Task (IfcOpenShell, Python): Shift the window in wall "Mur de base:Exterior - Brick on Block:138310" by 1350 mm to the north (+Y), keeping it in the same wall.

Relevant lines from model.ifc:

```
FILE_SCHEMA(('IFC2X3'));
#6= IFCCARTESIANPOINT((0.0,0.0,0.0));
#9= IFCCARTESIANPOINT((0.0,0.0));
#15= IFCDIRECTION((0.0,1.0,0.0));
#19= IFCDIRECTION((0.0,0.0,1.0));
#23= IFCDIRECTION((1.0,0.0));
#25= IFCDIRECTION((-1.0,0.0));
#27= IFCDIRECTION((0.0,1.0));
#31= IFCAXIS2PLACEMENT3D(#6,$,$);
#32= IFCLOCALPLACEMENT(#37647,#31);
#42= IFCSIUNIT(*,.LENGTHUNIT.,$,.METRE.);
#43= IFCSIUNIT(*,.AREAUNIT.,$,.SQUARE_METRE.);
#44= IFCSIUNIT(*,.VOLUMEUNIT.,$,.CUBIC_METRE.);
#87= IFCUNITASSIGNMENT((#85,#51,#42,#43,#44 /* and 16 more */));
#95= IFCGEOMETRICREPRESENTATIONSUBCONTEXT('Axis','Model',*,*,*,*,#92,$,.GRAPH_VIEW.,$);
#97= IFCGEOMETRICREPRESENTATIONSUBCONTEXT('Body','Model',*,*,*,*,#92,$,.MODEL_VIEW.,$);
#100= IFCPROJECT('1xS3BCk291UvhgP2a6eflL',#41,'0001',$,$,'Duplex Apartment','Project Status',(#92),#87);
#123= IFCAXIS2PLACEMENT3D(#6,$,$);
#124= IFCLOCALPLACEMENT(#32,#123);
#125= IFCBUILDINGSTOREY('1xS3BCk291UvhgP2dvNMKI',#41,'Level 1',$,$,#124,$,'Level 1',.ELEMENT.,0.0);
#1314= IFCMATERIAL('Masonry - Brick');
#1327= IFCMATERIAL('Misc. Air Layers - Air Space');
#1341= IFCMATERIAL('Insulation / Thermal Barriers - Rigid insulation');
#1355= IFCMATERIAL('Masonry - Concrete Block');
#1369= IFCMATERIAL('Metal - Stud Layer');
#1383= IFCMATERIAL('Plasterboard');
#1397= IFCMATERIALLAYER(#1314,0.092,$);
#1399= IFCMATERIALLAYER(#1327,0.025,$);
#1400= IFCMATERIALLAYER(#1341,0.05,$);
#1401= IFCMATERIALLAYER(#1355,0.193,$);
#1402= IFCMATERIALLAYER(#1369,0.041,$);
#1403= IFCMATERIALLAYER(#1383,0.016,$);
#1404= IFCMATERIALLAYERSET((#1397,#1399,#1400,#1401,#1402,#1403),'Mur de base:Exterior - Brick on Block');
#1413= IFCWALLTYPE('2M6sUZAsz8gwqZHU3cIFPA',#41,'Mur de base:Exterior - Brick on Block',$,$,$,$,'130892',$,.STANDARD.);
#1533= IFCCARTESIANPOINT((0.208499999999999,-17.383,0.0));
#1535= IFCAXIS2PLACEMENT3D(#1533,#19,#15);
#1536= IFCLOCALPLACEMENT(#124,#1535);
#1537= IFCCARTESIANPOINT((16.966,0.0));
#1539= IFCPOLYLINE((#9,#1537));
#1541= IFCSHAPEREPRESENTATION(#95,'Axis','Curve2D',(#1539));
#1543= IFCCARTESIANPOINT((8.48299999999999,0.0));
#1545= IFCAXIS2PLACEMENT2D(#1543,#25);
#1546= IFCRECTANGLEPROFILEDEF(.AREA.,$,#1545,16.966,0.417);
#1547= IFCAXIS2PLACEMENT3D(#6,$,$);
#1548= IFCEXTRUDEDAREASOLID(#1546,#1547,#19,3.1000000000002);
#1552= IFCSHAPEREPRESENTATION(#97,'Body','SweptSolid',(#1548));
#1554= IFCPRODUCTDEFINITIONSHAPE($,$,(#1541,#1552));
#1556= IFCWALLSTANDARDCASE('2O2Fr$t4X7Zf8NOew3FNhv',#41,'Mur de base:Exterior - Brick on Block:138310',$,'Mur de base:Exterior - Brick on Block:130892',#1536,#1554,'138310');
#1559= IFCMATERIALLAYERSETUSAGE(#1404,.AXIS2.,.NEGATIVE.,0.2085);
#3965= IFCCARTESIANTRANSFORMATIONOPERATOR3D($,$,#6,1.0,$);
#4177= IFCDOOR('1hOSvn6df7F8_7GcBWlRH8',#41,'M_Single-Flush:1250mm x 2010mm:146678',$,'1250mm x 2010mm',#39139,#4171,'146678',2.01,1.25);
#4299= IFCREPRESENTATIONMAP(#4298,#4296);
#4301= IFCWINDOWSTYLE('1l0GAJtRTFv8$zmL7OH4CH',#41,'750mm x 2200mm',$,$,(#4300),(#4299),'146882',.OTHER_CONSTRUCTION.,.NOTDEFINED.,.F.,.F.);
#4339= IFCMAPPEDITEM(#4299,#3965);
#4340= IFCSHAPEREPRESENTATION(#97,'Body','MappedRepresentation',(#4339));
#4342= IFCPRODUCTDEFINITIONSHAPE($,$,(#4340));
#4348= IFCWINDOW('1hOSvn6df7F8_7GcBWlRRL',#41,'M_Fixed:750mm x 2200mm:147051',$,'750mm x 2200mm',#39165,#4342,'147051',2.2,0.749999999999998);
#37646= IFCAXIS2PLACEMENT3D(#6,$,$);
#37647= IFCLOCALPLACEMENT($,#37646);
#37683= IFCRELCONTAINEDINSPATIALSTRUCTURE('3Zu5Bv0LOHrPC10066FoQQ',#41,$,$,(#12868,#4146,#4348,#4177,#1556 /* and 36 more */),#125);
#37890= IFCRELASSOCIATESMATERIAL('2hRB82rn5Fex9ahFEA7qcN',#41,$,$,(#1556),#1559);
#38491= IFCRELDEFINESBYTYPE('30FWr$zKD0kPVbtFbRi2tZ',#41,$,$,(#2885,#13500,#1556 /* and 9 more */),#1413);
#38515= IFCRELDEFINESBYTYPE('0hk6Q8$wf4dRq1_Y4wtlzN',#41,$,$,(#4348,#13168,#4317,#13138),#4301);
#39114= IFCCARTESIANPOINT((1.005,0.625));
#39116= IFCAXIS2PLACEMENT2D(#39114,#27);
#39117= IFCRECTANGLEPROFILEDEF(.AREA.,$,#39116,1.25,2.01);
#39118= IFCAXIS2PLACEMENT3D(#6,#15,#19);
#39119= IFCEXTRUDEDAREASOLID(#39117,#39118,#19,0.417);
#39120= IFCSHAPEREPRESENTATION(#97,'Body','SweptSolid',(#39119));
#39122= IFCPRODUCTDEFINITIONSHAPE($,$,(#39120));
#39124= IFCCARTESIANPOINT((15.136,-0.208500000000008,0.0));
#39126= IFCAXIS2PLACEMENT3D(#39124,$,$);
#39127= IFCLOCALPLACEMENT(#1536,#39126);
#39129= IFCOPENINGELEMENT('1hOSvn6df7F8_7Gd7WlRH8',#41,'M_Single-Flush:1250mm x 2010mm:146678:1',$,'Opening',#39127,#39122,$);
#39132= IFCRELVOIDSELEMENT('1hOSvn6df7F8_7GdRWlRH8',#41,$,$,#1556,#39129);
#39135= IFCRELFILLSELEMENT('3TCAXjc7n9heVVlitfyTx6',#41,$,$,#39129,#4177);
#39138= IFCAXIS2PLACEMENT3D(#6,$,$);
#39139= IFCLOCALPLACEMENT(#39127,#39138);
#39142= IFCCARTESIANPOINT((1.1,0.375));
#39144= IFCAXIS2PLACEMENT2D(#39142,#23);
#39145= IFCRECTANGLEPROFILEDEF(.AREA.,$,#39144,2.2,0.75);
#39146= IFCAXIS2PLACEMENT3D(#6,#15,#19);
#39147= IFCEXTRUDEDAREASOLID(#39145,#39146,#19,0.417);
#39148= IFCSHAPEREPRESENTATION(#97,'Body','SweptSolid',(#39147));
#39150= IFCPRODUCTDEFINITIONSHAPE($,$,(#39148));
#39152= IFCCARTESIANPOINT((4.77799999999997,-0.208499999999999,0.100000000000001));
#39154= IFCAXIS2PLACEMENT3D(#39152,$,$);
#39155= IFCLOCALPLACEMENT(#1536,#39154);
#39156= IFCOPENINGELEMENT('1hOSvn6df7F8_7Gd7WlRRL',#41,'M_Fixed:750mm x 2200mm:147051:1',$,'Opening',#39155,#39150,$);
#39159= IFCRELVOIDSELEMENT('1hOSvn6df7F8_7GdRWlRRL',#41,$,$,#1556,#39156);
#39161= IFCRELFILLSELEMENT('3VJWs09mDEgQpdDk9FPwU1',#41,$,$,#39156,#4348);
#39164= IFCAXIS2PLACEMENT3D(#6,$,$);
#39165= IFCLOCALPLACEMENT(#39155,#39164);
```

```python
import ifcopenshell
import ifcopenshell.api.geometry
import ifcopenshell.util.placement

model = ifcopenshell.open("model.ifc")

window = model.by_guid("1hOSvn6df7F8_7GcBWlRRL")
opening = window.FillsVoids[0].RelatingOpeningElement
wall = opening.VoidsElements[0].RelatingBuildingElement

wall_matrix = ifcopenshell.util.placement.get_local_placement(wall.ObjectPlacement)
shift = wall_matrix[:3, 0] * 1.35
before = ifcopenshell.util.placement.get_local_placement(window.ObjectPlacement)[:3, 3].copy()

# The window is placed relative to its opening, so it follows when the opening moves.
matrix = ifcopenshell.util.placement.get_local_placement(opening.ObjectPlacement)
matrix[:3, 3] += shift
ifcopenshell.api.geometry.edit_object_placement(
    model, product=opening, matrix=matrix, is_si=False, should_transform_children=True
)

after = ifcopenshell.util.placement.get_local_placement(window.ObjectPlacement)[:3, 3]
print("window moved by", (after - before).round(3) + 0.0)

model.write("model_updated.ifc")
```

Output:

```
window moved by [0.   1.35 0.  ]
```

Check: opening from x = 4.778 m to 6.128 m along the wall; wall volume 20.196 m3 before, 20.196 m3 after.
